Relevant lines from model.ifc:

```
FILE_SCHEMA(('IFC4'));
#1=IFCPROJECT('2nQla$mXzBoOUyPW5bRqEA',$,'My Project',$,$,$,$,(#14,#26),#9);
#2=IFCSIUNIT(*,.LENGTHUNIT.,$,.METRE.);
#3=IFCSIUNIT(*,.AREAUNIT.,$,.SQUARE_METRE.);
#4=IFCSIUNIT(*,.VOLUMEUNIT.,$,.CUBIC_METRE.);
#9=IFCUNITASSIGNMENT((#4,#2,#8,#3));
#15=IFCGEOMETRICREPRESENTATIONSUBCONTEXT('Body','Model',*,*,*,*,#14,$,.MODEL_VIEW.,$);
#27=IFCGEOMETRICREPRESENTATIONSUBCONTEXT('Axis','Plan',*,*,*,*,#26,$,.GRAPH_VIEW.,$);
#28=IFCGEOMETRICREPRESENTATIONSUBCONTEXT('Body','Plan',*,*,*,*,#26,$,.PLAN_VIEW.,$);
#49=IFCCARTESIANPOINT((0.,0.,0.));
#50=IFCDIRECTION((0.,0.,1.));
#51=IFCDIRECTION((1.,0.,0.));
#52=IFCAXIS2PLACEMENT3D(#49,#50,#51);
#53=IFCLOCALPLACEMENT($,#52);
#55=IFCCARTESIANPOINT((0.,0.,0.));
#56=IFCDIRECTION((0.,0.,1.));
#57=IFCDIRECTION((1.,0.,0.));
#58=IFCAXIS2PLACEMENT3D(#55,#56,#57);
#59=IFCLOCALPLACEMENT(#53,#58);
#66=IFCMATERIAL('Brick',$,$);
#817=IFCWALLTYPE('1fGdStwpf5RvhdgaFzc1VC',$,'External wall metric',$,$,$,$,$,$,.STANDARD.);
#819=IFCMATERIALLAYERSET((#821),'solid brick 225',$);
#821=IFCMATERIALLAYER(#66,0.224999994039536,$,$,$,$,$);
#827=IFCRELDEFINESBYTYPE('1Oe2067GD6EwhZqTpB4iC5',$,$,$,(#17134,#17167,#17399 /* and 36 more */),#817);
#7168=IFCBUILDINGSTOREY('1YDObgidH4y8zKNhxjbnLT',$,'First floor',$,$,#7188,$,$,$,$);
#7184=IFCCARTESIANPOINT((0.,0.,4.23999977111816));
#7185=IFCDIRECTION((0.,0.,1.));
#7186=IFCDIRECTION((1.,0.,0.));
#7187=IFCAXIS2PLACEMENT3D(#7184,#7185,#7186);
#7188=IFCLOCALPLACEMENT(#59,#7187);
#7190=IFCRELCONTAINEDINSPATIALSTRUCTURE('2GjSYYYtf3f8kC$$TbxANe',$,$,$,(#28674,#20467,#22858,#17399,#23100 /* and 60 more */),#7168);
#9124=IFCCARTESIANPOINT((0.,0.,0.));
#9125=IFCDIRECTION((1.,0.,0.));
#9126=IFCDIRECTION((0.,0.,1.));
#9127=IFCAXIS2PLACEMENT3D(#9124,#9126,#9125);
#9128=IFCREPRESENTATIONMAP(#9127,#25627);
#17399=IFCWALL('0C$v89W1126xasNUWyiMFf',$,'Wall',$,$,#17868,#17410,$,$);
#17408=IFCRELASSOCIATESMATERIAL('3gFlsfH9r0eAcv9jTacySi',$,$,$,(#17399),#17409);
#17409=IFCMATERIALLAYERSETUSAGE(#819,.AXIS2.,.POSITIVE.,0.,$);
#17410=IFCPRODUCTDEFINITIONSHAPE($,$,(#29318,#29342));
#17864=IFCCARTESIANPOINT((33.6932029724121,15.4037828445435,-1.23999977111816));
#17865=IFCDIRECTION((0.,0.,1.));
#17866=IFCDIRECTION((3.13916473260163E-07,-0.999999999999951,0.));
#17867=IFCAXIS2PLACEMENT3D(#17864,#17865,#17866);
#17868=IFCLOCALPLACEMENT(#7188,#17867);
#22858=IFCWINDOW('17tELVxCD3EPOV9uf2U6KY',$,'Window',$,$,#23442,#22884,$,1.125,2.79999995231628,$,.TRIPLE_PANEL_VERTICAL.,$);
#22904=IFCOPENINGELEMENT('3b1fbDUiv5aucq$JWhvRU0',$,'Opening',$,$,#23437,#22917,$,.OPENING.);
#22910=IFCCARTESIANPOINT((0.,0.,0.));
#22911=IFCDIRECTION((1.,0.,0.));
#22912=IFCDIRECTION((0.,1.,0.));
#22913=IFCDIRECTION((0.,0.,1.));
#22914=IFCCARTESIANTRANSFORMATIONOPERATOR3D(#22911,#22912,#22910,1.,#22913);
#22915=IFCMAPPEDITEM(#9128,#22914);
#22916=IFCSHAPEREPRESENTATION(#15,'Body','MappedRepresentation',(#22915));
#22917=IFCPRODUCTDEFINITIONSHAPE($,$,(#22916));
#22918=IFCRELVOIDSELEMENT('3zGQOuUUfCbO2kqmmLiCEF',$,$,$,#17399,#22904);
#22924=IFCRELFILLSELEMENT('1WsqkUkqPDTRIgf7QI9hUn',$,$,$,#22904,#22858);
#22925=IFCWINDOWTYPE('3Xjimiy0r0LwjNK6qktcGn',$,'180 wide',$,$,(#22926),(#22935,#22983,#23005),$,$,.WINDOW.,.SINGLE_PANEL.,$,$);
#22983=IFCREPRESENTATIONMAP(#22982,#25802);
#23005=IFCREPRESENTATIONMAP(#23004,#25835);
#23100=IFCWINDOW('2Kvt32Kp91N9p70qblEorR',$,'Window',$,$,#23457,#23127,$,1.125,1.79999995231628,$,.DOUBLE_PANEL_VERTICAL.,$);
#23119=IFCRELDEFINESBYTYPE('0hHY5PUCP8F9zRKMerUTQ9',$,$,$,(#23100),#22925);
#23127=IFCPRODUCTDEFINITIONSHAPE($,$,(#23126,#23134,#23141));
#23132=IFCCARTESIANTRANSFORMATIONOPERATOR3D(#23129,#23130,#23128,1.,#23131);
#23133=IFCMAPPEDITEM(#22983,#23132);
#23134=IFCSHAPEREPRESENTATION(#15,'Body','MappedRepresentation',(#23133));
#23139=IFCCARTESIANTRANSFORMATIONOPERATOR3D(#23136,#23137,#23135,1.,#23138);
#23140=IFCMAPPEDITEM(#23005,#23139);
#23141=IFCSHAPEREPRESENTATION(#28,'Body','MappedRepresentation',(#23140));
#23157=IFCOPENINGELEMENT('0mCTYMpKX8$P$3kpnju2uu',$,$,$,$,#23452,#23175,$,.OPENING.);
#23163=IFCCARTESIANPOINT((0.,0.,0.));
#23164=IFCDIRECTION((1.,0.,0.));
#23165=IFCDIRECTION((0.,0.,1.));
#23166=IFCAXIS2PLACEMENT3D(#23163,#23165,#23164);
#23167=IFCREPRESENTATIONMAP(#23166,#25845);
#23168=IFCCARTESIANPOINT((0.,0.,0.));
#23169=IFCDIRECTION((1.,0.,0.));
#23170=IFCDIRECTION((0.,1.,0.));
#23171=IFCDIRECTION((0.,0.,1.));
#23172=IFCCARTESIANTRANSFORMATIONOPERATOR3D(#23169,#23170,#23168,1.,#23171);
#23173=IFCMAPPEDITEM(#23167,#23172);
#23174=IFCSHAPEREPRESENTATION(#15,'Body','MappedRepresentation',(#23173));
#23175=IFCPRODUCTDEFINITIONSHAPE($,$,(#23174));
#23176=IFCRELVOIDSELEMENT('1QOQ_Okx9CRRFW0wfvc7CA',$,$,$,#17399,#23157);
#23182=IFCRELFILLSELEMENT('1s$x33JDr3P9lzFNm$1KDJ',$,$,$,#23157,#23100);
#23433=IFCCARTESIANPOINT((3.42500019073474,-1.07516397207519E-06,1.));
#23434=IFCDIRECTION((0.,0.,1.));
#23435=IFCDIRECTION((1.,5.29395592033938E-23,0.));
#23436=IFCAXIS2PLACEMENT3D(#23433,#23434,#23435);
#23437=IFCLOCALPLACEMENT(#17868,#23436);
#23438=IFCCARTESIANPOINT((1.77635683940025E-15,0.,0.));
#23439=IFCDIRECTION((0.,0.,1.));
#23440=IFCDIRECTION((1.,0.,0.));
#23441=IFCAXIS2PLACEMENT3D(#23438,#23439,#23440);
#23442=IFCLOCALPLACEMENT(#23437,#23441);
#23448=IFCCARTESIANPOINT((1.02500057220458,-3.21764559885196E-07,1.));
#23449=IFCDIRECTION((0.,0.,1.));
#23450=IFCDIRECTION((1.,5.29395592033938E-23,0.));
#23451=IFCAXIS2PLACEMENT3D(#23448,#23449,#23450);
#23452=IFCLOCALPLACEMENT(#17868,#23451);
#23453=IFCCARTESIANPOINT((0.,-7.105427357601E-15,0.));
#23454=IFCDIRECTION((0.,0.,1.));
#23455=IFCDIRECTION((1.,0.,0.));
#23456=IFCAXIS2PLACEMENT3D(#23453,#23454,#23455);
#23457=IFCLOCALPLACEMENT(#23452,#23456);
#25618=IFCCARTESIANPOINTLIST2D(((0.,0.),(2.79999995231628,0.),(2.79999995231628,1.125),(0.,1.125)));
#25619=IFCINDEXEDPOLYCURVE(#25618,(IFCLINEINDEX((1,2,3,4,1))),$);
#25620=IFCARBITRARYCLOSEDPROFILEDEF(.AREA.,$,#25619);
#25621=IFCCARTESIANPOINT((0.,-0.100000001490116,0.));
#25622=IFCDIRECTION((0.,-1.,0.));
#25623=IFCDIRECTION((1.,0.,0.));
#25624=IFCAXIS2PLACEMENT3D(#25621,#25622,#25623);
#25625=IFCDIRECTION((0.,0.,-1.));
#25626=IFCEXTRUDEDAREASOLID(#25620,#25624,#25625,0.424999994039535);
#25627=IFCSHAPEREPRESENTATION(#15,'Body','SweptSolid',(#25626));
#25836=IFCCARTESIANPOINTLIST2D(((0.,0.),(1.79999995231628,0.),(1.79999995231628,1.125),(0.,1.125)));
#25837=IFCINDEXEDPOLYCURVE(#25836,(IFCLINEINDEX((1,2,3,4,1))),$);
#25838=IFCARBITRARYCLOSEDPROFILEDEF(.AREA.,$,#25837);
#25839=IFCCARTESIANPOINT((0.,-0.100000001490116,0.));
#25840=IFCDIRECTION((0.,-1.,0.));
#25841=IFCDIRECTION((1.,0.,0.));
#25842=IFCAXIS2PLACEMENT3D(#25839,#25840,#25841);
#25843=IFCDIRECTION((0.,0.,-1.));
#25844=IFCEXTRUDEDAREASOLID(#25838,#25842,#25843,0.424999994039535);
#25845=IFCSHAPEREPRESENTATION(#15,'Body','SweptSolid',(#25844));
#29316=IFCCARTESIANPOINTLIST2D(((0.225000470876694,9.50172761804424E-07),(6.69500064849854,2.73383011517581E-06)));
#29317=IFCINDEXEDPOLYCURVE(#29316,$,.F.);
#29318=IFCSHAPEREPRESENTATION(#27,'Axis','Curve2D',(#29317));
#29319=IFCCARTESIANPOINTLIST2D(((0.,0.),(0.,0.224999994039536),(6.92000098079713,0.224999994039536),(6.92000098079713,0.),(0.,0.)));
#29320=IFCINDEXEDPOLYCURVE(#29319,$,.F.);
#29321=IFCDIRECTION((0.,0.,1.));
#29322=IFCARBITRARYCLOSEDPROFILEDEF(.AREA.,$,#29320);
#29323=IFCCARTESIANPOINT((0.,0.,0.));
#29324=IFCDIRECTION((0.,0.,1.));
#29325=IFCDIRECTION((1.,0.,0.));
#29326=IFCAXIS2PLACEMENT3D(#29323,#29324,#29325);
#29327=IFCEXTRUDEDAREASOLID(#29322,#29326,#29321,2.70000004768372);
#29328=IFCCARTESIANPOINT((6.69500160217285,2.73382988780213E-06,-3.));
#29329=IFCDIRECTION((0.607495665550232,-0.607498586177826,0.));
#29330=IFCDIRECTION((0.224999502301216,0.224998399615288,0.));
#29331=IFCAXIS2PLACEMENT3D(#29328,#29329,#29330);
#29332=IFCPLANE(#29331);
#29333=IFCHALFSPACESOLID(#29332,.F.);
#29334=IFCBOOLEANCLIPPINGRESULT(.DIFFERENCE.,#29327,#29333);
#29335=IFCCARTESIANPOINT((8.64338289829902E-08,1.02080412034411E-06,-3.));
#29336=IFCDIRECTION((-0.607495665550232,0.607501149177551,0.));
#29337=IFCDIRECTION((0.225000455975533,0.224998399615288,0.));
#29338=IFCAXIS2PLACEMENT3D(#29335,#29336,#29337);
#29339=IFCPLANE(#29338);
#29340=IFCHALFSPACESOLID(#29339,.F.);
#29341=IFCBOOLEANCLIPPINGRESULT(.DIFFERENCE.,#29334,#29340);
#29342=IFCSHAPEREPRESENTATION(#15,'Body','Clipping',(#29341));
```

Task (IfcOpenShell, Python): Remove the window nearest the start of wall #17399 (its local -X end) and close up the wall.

```python
import ifcopenshell
import ifcopenshell.api.feature
import ifcopenshell.api.root
import ifcopenshell.geom
import ifcopenshell.util.shape

model = ifcopenshell.open("model.ifc")
settings = ifcopenshell.geom.settings()


def volume(element):
    """Net volume in cubic metres, openings subtracted."""
    shape = ifcopenshell.geom.create_shape(settings, element)
    return ifcopenshell.util.shape.get_volume(shape.geometry)


window = model.by_id(23100)
opening = window.FillsVoids[0].RelatingOpeningElement
wall = opening.VoidsElements[0].RelatingBuildingElement
before = volume(wall)

ifcopenshell.api.root.remove_product(model, product=window)
ifcopenshell.api.feature.remove_feature(model, feature=opening)

after = volume(wall)

print(f"wall volume {before:.3f} -> {after:.3f} m3")

model.write("model_edited.ifc")
```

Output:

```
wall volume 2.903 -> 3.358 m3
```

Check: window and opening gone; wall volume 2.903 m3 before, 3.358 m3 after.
